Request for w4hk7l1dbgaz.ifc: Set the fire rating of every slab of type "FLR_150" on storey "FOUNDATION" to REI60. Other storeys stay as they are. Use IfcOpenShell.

First a look at what the model holds.

```python
import ifcopenshell
import ifcopenshell.util.element

model = ifcopenshell.open("w4hk7l1dbgaz.ifc")
print(model.schema)
storey = next(s for s in model.by_type("IfcBuildingStorey") if s.Name == "FOUNDATION")
slabs = [e for e in ifcopenshell.util.element.get_decomposition(storey) if e.is_a("IfcSlab")]
seen = {}
for e in slabs:
    element_type = ifcopenshell.util.element.get_type(e)
    key = (element_type.Name if element_type != e and element_type else None, ifcopenshell.util.element.get_pset(e, "Pset_SlabCommon", "FireRating"))
    seen[key] = seen.get(key, 0) + 1
for (name, value), count in sorted(seen.items(), key=str):
    print(count, "x", name, "|", value)
```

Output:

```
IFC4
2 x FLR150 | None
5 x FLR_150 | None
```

```python
import ifcopenshell
import ifcopenshell.api.pset
import ifcopenshell.util.element

model = ifcopenshell.open("w4hk7l1dbgaz.ifc")

storey = next(s for s in model.by_type("IfcBuildingStorey") if s.Name == "FOUNDATION")
slabs = [e for e in ifcopenshell.util.element.get_decomposition(storey) if e.is_a("IfcSlab")]

count = 0
for e in slabs:
    element_type = ifcopenshell.util.element.get_type(e)
    if element_type in (None, e) or element_type.Name != "FLR_150":
        continue
    # add_pset returns the element's existing set when there is one.
    pset = ifcopenshell.api.pset.add_pset(model, product=e, name="Pset_SlabCommon")
    ifcopenshell.api.pset.edit_pset(model, pset=pset, properties={"FireRating": "REI60"})
    count += 1

print(count, "slabs updated")

model.write("w4hk7l1dbgaz-out.ifc")
```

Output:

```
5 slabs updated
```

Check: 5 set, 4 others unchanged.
